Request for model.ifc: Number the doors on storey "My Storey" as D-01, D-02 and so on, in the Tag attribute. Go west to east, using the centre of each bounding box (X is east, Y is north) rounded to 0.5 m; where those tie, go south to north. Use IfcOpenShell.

First a look at what the model holds.

```python
import ifcopenshell
import ifcopenshell.util.element
import ifcopenshell.util.placement

model = ifcopenshell.open("model.ifc")
print(model.schema)
storey = next(s for s in model.by_type("IfcBuildingStorey") if s.Name == "My Storey")
doors = [e for e in ifcopenshell.util.element.get_decomposition(storey) if e.is_a("IfcDoor")]
for e in sorted(doors, key=lambda e: e.id()):
    origin = ifcopenshell.util.placement.get_local_placement(e.ObjectPlacement)[:3, 3]
    print(e.id(), e.Tag, e.Name, origin.round(2) + 0.0, sep=" | ")
```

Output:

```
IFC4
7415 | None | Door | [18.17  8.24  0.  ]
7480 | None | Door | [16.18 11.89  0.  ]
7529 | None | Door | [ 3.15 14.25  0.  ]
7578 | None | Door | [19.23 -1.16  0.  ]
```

```python
import ifcopenshell
import ifcopenshell.geom
import ifcopenshell.util.element
import ifcopenshell.util.shape

model = ifcopenshell.open("model.ifc")
settings = ifcopenshell.geom.settings()
settings.set("use-world-coords", True)


def centre(element):
    shape = ifcopenshell.geom.create_shape(settings, element)
    return ifcopenshell.util.shape.get_bbox_centroid(shape.geometry)


storey = next(s for s in model.by_type("IfcBuildingStorey") if s.Name == "My Storey")
doors = [e for e in ifcopenshell.util.element.get_decomposition(storey) if e.is_a("IfcDoor")]

# Insertion points can sit at a corner or the storey origin, so sort by the geometry (in metres).
centres = {e: centre(e) for e in doors}
doors.sort(key=lambda e: (round(centres[e][0] / 0.5), centres[e][1]))

for i, e in enumerate(doors, start=1):
    number = f"D-{i:02d}"
    e.Tag = number
    print(e.id(), number)

model.write("model-out.ifc")
```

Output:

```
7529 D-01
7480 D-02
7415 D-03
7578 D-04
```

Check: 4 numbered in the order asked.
